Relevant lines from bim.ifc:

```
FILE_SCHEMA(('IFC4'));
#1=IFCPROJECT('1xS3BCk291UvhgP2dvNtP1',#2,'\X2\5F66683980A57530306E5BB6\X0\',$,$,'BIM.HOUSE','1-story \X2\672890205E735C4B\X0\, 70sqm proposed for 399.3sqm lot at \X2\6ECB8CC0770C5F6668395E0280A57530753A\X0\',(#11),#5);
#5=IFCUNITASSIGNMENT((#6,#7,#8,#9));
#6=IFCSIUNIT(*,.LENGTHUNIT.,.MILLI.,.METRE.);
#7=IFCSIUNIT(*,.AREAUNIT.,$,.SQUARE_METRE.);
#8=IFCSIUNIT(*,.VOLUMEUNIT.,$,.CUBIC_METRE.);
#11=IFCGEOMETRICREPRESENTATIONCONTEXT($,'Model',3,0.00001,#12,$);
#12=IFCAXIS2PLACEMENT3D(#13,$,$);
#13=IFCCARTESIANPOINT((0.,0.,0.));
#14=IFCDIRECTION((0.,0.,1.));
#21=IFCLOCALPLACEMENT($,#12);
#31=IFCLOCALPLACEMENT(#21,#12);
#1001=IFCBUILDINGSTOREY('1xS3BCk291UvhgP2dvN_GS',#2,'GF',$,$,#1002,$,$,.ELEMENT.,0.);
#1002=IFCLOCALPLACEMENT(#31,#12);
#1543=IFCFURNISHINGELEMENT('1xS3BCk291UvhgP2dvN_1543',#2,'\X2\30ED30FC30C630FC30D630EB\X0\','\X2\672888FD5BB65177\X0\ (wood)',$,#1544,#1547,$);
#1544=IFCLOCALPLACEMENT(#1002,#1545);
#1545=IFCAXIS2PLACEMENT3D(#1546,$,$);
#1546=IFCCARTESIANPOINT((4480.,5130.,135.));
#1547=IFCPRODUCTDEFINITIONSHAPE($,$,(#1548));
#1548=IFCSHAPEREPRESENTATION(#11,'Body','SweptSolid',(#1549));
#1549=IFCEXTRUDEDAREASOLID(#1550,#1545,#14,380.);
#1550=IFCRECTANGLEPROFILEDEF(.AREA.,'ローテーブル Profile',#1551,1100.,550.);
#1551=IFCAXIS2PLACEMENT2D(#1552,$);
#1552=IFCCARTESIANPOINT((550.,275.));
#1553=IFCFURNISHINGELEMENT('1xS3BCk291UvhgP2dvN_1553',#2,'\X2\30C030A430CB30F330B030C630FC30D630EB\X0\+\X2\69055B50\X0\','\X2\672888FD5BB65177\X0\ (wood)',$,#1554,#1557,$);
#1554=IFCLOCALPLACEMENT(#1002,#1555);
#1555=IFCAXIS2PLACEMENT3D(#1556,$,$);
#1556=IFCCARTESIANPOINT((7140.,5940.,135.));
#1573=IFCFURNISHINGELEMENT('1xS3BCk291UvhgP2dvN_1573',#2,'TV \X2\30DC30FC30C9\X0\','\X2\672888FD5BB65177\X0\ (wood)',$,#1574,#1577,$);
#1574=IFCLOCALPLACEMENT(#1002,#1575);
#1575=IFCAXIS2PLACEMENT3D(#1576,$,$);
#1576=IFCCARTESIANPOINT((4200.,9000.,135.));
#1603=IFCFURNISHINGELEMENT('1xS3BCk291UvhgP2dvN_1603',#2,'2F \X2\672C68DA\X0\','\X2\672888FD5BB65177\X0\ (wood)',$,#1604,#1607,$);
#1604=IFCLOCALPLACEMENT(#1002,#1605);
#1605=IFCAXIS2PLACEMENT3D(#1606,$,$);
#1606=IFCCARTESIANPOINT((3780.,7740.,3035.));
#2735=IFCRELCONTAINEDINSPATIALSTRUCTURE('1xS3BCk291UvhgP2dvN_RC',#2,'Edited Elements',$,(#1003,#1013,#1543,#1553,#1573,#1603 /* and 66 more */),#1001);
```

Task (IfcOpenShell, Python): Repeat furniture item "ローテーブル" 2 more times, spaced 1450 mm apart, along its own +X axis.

```python
import ifcopenshell
import ifcopenshell.api.geometry
import ifcopenshell.api.root
import ifcopenshell.util.element
import ifcopenshell.util.placement
import ifcopenshell.util.unit

model = ifcopenshell.open("bim.ifc")
unit_scale = ifcopenshell.util.unit.calculate_unit_scale(model)


def reuse_history(source, copy):
    """copy_class also copies each property set's owner history, people and application; keep the originals."""
    for rel in copy.IsDefinedBy:
        if rel.is_a("IfcRelDefinesByProperties") and (history := rel.RelatingPropertyDefinition.OwnerHistory):
            rel.RelatingPropertyDefinition.OwnerHistory = source.OwnerHistory
            ifcopenshell.util.element.remove_deep2(model, history)


source = model.by_guid("1xS3BCk291UvhgP2dvN_1543")
base = ifcopenshell.util.placement.get_local_placement(source.ObjectPlacement)
step = base[:3, 0] * 1.45 / unit_scale

for i in range(1, 3):
    copy = ifcopenshell.api.root.copy_class(model, product=source)
    copy.Representation = ifcopenshell.util.element.copy_deep(
        model, source.Representation, exclude=["IfcGeometricRepresentationContext", "IfcRepresentationMap"]
    )
    reuse_history(source, copy)
    matrix = base.copy()
    matrix[:3, 3] += i * step
    print("added at", matrix[:3, 3].round(3) + 0.0)
    ifcopenshell.api.geometry.edit_object_placement(model, product=copy, matrix=matrix, is_si=False)

model.write("bim_rev.ifc")
```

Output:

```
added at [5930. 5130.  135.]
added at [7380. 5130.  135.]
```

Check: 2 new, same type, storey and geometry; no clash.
